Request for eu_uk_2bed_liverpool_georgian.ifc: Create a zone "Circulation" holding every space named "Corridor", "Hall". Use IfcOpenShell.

First a look at what the model holds.

```python
import ifcopenshell

model = ifcopenshell.open("eu_uk_2bed_liverpool_georgian.ifc")
print(model.schema)
seen = {}
for space in model.by_type("IfcSpace"):
    seen[space.LongName] = seen.get(space.LongName, 0) + 1
for name, count in sorted(seen.items(), key=str):
    print(count, "x", name)
print("zones:", [z.Name for z in model.by_type("IfcZone")][:20])
```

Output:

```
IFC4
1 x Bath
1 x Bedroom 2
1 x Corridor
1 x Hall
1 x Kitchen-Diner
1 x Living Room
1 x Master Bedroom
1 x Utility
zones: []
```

```python
import ifcopenshell
import ifcopenshell.api.group
import ifcopenshell.api.root

model = ifcopenshell.open("eu_uk_2bed_liverpool_georgian.ifc")

names = {"Corridor", "Hall"}
spaces = [s for s in model.by_type("IfcSpace") if s.LongName in names]

zone = ifcopenshell.api.root.create_entity(model, ifc_class="IfcZone", name="Circulation")
ifcopenshell.api.group.assign_group(model, products=spaces, group=zone)
print(len(spaces), "spaces in", zone.Name)

model.write("eu_uk_2bed_liverpool_georgian_updated.ifc")
```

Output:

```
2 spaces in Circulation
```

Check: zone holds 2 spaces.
